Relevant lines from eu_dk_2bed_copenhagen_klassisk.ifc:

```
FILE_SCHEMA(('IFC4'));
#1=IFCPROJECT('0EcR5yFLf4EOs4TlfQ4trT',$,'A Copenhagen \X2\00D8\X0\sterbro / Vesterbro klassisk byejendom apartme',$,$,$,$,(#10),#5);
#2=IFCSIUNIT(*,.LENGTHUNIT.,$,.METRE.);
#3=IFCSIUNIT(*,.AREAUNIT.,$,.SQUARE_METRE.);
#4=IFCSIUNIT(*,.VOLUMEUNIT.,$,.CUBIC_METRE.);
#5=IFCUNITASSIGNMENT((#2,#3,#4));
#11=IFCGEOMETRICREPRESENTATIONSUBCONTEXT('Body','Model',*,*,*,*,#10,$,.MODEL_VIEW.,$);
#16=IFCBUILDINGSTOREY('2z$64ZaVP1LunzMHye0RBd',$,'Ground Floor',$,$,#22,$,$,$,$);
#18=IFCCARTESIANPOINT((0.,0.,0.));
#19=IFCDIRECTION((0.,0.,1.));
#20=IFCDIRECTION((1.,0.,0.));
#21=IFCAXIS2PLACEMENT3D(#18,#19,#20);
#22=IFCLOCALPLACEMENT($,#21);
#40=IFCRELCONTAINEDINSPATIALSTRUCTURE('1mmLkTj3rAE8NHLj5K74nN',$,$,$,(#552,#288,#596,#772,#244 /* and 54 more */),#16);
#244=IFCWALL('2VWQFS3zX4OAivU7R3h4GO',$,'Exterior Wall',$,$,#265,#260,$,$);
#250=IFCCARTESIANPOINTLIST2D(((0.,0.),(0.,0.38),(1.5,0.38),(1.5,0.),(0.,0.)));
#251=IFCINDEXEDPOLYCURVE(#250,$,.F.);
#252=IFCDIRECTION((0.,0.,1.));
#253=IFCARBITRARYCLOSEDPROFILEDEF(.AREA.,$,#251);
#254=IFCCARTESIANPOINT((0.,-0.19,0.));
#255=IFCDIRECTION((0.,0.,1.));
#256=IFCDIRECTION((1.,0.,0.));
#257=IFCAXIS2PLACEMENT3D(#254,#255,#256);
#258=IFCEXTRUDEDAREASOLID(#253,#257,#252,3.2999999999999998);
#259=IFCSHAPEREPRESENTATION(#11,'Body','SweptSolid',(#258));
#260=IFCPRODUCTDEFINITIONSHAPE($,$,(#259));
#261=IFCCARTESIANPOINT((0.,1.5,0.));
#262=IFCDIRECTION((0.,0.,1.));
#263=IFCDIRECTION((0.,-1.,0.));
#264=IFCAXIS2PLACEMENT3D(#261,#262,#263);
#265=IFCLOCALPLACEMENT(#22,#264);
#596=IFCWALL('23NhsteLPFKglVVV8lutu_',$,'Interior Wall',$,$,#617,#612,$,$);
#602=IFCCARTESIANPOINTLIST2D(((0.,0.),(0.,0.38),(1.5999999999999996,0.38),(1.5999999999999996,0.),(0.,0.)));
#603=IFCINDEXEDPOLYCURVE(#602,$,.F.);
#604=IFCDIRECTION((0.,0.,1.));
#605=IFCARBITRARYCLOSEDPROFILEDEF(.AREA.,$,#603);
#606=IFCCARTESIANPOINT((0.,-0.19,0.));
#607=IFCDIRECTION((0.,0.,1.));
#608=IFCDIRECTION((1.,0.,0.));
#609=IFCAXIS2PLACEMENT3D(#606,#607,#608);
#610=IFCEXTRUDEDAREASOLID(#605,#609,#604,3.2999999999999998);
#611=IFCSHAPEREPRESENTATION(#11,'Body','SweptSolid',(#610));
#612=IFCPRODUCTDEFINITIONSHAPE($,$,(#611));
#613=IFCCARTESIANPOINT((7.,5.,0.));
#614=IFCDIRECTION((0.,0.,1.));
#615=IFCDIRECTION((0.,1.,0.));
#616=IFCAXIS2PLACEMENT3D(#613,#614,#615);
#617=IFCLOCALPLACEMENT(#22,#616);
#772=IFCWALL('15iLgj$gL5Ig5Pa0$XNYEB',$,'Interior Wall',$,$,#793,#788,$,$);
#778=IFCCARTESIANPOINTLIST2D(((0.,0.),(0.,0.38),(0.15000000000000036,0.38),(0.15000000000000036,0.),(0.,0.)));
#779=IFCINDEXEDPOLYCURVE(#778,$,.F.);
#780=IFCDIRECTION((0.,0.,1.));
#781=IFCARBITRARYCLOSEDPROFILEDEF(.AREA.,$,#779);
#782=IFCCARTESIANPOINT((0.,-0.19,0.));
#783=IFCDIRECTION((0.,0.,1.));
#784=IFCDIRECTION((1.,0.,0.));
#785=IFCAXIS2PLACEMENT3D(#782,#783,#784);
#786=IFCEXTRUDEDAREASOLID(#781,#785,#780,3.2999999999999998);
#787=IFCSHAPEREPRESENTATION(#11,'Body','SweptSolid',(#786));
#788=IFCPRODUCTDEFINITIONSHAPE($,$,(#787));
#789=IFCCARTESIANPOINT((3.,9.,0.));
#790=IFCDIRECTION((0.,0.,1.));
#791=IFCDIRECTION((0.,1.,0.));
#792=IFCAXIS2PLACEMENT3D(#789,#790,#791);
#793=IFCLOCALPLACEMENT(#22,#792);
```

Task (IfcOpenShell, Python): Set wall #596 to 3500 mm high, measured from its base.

```python
import ifcopenshell
import ifcopenshell.geom
import ifcopenshell.util.representation
import ifcopenshell.util.shape
import ifcopenshell.util.unit

model = ifcopenshell.open("eu_dk_2bed_copenhagen_klassisk.ifc")
unit_scale = ifcopenshell.util.unit.calculate_unit_scale(model)
settings = ifcopenshell.geom.settings()


def volume(element):
    """Net volume in cubic metres, openings subtracted."""
    shape = ifcopenshell.geom.create_shape(settings, element)
    return ifcopenshell.util.shape.get_volume(shape.geometry)


wall = model.by_id(596)
before = volume(wall)

body = ifcopenshell.util.representation.get_representation(wall, "Model", "Body")
solid = body.Items[0]
old_height = solid.Depth
solid.Depth = 3.5 / unit_scale
after = volume(wall)

print(f"height {old_height:g} -> {solid.Depth:g}, volume {before:.3f} -> {after:.3f} m3")

model.write("eu_dk_2bed_copenhagen_klassisk_updated.ifc")
```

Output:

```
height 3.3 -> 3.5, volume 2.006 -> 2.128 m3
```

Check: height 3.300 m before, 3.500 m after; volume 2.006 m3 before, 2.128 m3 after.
